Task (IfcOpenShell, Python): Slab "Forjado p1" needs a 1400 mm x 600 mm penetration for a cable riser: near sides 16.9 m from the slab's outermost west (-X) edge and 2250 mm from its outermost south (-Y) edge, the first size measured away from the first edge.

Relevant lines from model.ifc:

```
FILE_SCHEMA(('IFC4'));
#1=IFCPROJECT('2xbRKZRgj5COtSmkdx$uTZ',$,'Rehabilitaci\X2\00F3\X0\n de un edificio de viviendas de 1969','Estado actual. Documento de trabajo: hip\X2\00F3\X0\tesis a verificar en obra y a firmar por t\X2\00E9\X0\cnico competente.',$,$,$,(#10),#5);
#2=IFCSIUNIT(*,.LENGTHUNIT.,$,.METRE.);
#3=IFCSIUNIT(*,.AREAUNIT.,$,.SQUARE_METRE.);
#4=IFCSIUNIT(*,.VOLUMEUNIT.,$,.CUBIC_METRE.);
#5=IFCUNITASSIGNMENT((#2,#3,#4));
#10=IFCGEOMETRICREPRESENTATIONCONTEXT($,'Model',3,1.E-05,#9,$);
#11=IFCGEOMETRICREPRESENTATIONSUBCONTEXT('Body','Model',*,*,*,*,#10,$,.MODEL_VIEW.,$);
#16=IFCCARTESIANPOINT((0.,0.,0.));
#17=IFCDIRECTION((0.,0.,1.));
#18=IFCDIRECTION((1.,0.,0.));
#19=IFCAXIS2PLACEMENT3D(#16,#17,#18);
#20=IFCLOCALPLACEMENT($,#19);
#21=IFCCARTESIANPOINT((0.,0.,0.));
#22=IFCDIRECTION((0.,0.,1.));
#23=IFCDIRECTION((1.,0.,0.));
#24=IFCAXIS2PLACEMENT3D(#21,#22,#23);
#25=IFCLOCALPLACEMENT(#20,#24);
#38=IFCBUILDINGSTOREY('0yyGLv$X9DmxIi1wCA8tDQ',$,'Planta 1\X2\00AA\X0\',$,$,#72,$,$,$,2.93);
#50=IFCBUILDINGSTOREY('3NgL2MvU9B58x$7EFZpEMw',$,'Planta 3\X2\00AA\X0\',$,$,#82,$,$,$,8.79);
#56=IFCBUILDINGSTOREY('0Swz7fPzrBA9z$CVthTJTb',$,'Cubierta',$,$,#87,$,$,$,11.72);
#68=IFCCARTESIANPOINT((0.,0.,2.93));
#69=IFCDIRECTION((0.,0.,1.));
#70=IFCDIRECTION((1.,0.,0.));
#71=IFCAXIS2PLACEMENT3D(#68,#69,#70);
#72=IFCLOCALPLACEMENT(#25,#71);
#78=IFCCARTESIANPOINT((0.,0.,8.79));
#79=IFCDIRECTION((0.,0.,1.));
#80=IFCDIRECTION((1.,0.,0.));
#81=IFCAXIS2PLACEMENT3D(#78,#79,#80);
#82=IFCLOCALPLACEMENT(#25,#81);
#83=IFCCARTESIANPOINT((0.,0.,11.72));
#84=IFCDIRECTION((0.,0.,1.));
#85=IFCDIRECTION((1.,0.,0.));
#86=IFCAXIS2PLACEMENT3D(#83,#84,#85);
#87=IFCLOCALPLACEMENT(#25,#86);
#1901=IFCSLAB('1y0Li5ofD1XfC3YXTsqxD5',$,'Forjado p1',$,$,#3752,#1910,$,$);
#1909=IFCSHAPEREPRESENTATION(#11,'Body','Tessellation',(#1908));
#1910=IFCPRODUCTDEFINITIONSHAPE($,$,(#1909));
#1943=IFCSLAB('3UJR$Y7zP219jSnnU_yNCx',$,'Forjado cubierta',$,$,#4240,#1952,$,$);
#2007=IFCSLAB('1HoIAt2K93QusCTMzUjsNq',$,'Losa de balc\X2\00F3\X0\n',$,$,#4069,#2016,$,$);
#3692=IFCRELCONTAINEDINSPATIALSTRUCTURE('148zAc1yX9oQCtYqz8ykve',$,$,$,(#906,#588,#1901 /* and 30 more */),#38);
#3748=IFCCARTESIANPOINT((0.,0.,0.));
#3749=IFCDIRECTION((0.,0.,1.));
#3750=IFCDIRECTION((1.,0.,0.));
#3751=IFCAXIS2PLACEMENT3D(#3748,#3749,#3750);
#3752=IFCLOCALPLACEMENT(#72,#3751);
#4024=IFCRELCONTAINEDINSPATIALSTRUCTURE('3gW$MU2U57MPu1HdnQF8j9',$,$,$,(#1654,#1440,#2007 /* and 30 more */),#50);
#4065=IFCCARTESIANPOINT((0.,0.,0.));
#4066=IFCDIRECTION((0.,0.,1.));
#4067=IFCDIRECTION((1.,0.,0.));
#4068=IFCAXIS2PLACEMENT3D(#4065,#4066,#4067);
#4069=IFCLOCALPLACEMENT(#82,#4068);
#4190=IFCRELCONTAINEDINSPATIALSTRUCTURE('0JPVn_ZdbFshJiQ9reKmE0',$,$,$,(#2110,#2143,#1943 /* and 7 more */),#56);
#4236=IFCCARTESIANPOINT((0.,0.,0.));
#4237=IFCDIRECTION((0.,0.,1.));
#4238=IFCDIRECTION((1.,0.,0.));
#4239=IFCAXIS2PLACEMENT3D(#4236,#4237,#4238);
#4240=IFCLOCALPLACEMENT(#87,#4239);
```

```python
import numpy as np
import ifcopenshell
import ifcopenshell.api.feature
import ifcopenshell.api.geometry
import ifcopenshell.api.root
import ifcopenshell.geom
import ifcopenshell.util.placement
import ifcopenshell.util.representation
import ifcopenshell.util.shape
import ifcopenshell.util.unit

model = ifcopenshell.open("model.ifc")
unit_scale = ifcopenshell.util.unit.calculate_unit_scale(model)
settings = ifcopenshell.geom.settings()


def volume(element):
    """Net volume in cubic metres, openings subtracted."""
    shape = ifcopenshell.geom.create_shape(settings, element)
    return ifcopenshell.util.shape.get_volume(shape.geometry)


slab = model.by_guid("1y0Li5ofD1XfC3YXTsqxD5")
before = volume(slab)

# Extent in the slab's own axes, in metres. The edges named are its -X and -Y sides.
slab_shape = ifcopenshell.geom.create_shape(settings, slab)
vertices = ifcopenshell.util.shape.get_vertices(slab_shape.geometry)
x_min, y_min, bottom = vertices.min(axis=0)
top = vertices[:, 2].max()

opening = ifcopenshell.api.root.create_entity(model, ifc_class="IfcOpeningElement", name="Cable riser opening", predefined_type="OPENING")
context = ifcopenshell.util.representation.get_context(model, "Model", "Body", "MODEL_VIEW")
width, depth = 1.4, 0.6
outline = [(0.0, 0.0), (width, 0.0), (width, depth), (0.0, depth), (0.0, 0.0)]
# Overshoot both faces by 50 mm so the cut is clean.
shape = ifcopenshell.api.geometry.add_slab_representation(
    model, context=context, depth=top - bottom + 0.1, polyline=outline
)
ifcopenshell.api.geometry.assign_representation(model, product=opening, representation=shape)

matrix = ifcopenshell.util.placement.get_local_placement(slab.ObjectPlacement)
matrix[:, 3] = matrix @ np.append(np.array([x_min + 16.9, y_min + 2.25, bottom - 0.05]) / unit_scale, 1.0)
ifcopenshell.api.geometry.edit_object_placement(model, product=opening, matrix=matrix, is_si=False)
ifcopenshell.api.feature.add_feature(model, feature=opening, element=slab)

after = volume(slab)

print(f"slab volume {before:.3f} -> {after:.3f} m3")

model.write("model-out.ifc")
```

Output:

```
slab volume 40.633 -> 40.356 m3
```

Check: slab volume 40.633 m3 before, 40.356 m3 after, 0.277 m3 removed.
